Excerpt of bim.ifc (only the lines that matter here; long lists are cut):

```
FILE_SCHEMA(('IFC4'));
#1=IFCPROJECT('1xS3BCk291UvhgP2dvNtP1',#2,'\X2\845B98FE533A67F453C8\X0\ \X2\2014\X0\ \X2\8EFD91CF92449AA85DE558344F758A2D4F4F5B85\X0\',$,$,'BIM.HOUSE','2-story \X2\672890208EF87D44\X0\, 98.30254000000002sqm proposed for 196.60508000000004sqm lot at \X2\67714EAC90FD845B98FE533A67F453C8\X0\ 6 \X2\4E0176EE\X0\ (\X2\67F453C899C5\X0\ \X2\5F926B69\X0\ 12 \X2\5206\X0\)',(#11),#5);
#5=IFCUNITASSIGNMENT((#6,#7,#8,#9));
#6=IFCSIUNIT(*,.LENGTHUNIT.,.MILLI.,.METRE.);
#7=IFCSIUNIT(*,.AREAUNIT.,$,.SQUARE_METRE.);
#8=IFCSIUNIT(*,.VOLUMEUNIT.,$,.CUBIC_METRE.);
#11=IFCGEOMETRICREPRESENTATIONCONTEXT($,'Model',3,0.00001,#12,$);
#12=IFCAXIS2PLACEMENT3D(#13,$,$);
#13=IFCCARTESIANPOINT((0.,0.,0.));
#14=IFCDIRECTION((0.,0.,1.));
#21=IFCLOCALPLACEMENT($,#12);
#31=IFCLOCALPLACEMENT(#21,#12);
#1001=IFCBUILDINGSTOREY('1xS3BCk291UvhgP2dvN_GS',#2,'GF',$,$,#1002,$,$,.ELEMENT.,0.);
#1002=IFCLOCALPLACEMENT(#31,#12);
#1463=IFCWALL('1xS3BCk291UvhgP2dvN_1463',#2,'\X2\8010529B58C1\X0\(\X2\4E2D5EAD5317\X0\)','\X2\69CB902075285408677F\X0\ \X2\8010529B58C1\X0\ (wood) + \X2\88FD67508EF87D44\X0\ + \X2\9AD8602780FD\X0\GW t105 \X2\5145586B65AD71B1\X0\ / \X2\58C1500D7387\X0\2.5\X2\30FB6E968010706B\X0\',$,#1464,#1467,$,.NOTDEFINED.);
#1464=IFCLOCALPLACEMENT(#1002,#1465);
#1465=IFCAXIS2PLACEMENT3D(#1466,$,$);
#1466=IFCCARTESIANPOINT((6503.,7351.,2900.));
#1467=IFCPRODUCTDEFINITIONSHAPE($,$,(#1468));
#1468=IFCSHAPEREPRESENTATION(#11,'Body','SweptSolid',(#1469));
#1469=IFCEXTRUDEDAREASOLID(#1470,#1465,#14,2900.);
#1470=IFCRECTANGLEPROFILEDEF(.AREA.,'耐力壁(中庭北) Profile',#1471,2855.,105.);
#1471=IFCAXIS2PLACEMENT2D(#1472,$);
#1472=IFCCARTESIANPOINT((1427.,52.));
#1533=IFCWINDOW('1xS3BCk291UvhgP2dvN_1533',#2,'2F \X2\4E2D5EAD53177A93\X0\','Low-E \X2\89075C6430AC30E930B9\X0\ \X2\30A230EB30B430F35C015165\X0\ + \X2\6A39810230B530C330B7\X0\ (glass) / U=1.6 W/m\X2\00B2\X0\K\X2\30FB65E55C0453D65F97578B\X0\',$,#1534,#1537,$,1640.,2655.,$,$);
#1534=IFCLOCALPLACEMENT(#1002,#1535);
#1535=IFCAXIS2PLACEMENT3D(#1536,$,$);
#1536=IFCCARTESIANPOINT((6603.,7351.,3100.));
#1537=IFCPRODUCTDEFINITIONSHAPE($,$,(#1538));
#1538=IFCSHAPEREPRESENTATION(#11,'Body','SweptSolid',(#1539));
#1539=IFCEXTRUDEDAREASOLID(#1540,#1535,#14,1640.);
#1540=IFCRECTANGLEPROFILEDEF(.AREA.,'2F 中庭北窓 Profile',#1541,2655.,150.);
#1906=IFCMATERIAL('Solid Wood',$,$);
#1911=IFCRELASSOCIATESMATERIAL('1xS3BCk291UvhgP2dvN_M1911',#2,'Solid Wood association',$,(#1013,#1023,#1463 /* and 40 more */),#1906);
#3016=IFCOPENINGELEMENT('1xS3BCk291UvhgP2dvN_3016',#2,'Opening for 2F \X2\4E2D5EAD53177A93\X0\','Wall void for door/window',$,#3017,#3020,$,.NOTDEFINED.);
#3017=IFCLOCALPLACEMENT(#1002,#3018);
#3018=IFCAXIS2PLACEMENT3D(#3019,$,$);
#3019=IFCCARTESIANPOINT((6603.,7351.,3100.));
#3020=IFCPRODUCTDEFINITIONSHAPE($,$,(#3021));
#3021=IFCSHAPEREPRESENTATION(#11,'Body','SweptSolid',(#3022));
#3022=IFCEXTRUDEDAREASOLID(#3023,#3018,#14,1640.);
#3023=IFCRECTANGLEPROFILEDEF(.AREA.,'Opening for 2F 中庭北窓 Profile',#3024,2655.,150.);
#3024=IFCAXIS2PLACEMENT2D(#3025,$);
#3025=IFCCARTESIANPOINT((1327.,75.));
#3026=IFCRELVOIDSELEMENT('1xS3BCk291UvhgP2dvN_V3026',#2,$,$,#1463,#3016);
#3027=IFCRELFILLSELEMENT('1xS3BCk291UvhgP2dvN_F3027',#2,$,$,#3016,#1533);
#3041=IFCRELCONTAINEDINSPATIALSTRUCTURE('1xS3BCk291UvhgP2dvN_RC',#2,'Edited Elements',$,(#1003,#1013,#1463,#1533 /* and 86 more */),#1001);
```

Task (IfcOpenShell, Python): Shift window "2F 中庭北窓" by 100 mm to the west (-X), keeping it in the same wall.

```python
import ifcopenshell
import ifcopenshell.api.geometry
import ifcopenshell.util.placement
import ifcopenshell.util.unit

model = ifcopenshell.open("bim.ifc")
unit_scale = ifcopenshell.util.unit.calculate_unit_scale(model)

window = model.by_guid("1xS3BCk291UvhgP2dvN_1533")
opening = window.FillsVoids[0].RelatingOpeningElement
wall = opening.VoidsElements[0].RelatingBuildingElement

wall_matrix = ifcopenshell.util.placement.get_local_placement(wall.ObjectPlacement)
shift = wall_matrix[:3, 0] * -0.1 / unit_scale
before = ifcopenshell.util.placement.get_local_placement(window.ObjectPlacement)[:3, 3].copy()

# The window is not placed relative to its opening, so move both.
for product in (opening, window):
    matrix = ifcopenshell.util.placement.get_local_placement(product.ObjectPlacement)
    matrix[:3, 3] += shift
    ifcopenshell.api.geometry.edit_object_placement(model, product=product, matrix=matrix, is_si=False)

after = ifcopenshell.util.placement.get_local_placement(window.ObjectPlacement)[:3, 3]
print("window moved by", (after - before).round(3) + 0.0)

model.write("bim_v2.ifc")
```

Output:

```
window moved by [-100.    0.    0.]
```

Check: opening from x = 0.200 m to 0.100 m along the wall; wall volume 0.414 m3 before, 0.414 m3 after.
